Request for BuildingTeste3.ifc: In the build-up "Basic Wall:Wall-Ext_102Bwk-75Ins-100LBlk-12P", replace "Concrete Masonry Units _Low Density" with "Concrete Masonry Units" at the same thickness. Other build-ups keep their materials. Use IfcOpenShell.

First a look at what the model holds.

```python
import ifcopenshell
import ifcopenshell.util.element

model = ifcopenshell.open("BuildingTeste3.ifc")
print(model.schema)
for layer_set in model.by_type("IfcMaterialLayerSet"):
    if layer_set.LayerSetName == "Basic Wall:Wall-Ext_102Bwk-75Ins-100LBlk-12P":
        for layer in layer_set.MaterialLayers:
            print(layer.id(), layer.Material and layer.Material.Name, layer.LayerThickness, sep=" | ")
        print(len(ifcopenshell.util.element.get_elements_by_material(model, layer_set)), "elements and types use it")
print(sorted(m.Name for m in model.by_type("IfcMaterial") if m.Name)[:60])
```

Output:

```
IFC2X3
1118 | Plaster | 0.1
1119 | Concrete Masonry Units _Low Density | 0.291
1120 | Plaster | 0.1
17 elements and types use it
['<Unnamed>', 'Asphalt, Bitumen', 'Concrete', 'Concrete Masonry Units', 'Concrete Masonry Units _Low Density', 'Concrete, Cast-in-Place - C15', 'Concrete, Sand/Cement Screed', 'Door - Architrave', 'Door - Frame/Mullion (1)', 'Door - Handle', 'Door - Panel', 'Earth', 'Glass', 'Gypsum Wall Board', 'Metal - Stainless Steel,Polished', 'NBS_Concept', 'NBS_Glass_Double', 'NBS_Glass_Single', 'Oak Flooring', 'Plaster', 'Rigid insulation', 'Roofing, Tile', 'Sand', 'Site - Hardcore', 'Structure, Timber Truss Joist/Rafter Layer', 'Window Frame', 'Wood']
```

```python
import ifcopenshell
import ifcopenshell.api.material

model = ifcopenshell.open("BuildingTeste3.ifc")

layer_set = next(s for s in model.by_type("IfcMaterialLayerSet") if s.LayerSetName == "Basic Wall:Wall-Ext_102Bwk-75Ins-100LBlk-12P")
layer = next(l for l in layer_set.MaterialLayers if l.Material and l.Material.Name == "Concrete Masonry Units _Low Density")
material = next(m for m in model.by_type("IfcMaterial") if m.Name == "Concrete Masonry Units")

# Point this one layer at the other material; renaming the old one would change it everywhere.
ifcopenshell.api.material.edit_layer(model, layer=layer, attributes={}, material=material)

print([l.Material.Name if l.Material else None for l in layer_set.MaterialLayers])

model.write("BuildingTeste3_edited.ifc")
```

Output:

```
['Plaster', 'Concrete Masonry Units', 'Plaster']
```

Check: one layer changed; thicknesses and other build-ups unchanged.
